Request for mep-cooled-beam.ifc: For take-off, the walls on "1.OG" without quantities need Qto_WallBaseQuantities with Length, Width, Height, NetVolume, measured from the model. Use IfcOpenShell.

First a look at what the model holds.

```python
import ifcopenshell
import ifcopenshell.util.element
import ifcopenshell.util.unit

model = ifcopenshell.open("mep-cooled-beam.ifc")
print(model.schema)
for unit_type in ("LENGTHUNIT", "AREAUNIT", "VOLUMEUNIT"):
    print(unit_type, ifcopenshell.util.unit.calculate_unit_scale(model, unit_type))
storey = next(s for s in model.by_type("IfcBuildingStorey") if s.Name == "1.OG")
walls = [e for e in ifcopenshell.util.element.get_decomposition(storey) if e.is_a("IfcWall")]
for e in sorted(walls, key=lambda e: e.id()):
    print(e.id(), e.is_a(), e.Name, list(ifcopenshell.util.element.get_psets(e, qtos_only=True)), sep=" | ")
```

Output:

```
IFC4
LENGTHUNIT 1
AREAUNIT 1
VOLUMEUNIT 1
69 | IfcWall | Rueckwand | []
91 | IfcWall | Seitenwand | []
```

```python
import ifcopenshell
import ifcopenshell.api.pset
import ifcopenshell.geom
import ifcopenshell.util.element
import ifcopenshell.util.shape
import ifcopenshell.util.unit

model = ifcopenshell.open("mep-cooled-beam.ifc")
unit_scale = ifcopenshell.util.unit.calculate_unit_scale(model)
volume_scale = ifcopenshell.util.unit.calculate_unit_scale(model, "VOLUMEUNIT")
settings = ifcopenshell.geom.settings()

storey = next(s for s in model.by_type("IfcBuildingStorey") if s.Name == "1.OG")
walls = [e for e in ifcopenshell.util.element.get_decomposition(storey) if e.is_a("IfcWall")]

for e in sorted(walls, key=lambda e: e.id()):
    if ifcopenshell.util.element.get_psets(e, qtos_only=True, should_inherit=False):
        continue
    # Geometry comes back in metres, in the element's own axes.
    shape = ifcopenshell.geom.create_shape(settings, e)
    values = {
        "Length": ifcopenshell.util.shape.get_x(shape.geometry) / unit_scale,
        "Width": ifcopenshell.util.shape.get_y(shape.geometry) / unit_scale,
        "Height": ifcopenshell.util.shape.get_z(shape.geometry) / unit_scale,
        "NetVolume": ifcopenshell.util.shape.get_volume(shape.geometry) / volume_scale,
    }
    qto = ifcopenshell.api.pset.add_qto(model, product=e, name="Qto_WallBaseQuantities")
    ifcopenshell.api.pset.edit_qto(model, qto=qto, properties=values)
    print(e.id(), {k: round(v, 3) for k, v in values.items()})

model.write("mep-cooled-beam_v2.ifc")
```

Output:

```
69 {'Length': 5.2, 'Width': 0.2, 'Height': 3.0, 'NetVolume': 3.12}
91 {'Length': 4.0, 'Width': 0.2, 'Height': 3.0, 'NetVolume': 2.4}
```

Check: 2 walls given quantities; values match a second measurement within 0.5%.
